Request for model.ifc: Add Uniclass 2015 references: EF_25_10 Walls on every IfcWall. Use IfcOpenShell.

First a look at what the model holds.

```python
import ifcopenshell

model = ifcopenshell.open("model.ifc")
print(model.schema)
print("classifications:", [c.Name for c in model.by_type("IfcClassification")])
for ifc_class in ("IfcDoor", "IfcRoof", "IfcStair", "IfcWall", "IfcWindow"):
    print(ifc_class, len(model.by_type(ifc_class)))
```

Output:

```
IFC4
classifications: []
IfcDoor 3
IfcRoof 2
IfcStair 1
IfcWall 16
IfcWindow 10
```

```python
import ifcopenshell
import ifcopenshell.api.classification

model = ifcopenshell.open("model.ifc")

system = ifcopenshell.api.classification.add_classification(model, classification="Uniclass 2015")

codes = {
    "IfcWall": ("EF_25_10", "Walls"),
}
for ifc_class, (code, name) in codes.items():
    products = model.by_type(ifc_class)
    ifcopenshell.api.classification.add_reference(
        model, products=products, classification=system, identification=code, name=name
    )
    print(code, len(products))

model.write("model_rev.ifc")
```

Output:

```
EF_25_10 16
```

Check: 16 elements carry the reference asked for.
